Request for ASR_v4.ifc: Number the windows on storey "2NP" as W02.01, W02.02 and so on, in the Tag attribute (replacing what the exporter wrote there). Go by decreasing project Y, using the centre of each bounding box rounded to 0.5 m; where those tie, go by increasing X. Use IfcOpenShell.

First a look at what the model holds.

```python
import ifcopenshell
import ifcopenshell.util.element
import ifcopenshell.util.placement

model = ifcopenshell.open("ASR_v4.ifc")
print(model.schema)
storey = next(s for s in model.by_type("IfcBuildingStorey") if s.Name == "2NP")
windows = [e for e in ifcopenshell.util.element.get_decomposition(storey) if e.is_a("IfcWindow")]
for e in sorted(windows, key=lambda e: e.id()):
    origin = ifcopenshell.util.placement.get_local_placement(e.ObjectPlacement)[:3, 3]
    print(e.id(), e.Tag, e.Name, origin.round(2) + 0.0, sep=" | ")
```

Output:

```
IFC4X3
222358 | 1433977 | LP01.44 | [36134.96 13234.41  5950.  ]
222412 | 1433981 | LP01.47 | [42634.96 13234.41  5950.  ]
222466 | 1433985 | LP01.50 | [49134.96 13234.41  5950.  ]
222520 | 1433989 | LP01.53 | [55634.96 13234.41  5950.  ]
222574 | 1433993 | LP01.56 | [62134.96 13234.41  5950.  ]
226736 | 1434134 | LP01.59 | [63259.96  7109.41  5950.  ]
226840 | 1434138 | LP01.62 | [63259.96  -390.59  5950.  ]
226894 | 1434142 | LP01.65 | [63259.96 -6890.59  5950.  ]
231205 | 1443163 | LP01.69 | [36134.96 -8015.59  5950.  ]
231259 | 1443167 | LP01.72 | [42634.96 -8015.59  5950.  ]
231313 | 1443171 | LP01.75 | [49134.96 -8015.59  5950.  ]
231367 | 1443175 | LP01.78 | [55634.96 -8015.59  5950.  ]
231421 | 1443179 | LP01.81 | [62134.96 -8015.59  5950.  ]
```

```python
import ifcopenshell
import ifcopenshell.geom
import ifcopenshell.util.element
import ifcopenshell.util.shape

model = ifcopenshell.open("ASR_v4.ifc")
settings = ifcopenshell.geom.settings()
settings.set("use-world-coords", True)


def centre(element):
    shape = ifcopenshell.geom.create_shape(settings, element)
    return ifcopenshell.util.shape.get_bbox_centroid(shape.geometry)


storey = next(s for s in model.by_type("IfcBuildingStorey") if s.Name == "2NP")
windows = [e for e in ifcopenshell.util.element.get_decomposition(storey) if e.is_a("IfcWindow")]

# Insertion points can sit at a corner or the storey origin, so sort by the geometry (in metres).
centres = {e: centre(e) for e in windows}
windows.sort(key=lambda e: (-round(centres[e][1] / 0.5), centres[e][0]))

for i, e in enumerate(windows, start=1):
    number = f"W02.{i:02d}"
    e.Tag = number
    print(e.id(), number)

model.write("ASR_v4_rev.ifc")
```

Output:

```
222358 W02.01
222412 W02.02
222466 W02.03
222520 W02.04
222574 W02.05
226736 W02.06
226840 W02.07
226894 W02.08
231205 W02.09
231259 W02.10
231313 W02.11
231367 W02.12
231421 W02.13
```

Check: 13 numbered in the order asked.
